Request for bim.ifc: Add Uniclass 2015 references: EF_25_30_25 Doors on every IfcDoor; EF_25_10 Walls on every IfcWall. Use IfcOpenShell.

First a look at what the model holds.

```python
import ifcopenshell

model = ifcopenshell.open("bim.ifc")
print(model.schema)
print("classifications:", [c.Name for c in model.by_type("IfcClassification")])
for ifc_class in ("IfcDoor", "IfcRoof", "IfcStair", "IfcWall", "IfcWindow"):
    print(ifc_class, len(model.by_type(ifc_class)))
```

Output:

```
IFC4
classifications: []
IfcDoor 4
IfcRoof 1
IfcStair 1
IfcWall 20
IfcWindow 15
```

```python
import ifcopenshell
import ifcopenshell.api.classification

model = ifcopenshell.open("bim.ifc")

system = ifcopenshell.api.classification.add_classification(model, classification="Uniclass 2015")

codes = {
    "IfcDoor": ("EF_25_30_25", "Doors"),
    "IfcWall": ("EF_25_10", "Walls"),
}
for ifc_class, (code, name) in codes.items():
    products = model.by_type(ifc_class)
    ifcopenshell.api.classification.add_reference(
        model, products=products, classification=system, identification=code, name=name
    )
    print(code, len(products))

model.write("bim_edited.ifc")
```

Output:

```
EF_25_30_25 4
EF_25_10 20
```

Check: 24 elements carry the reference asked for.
